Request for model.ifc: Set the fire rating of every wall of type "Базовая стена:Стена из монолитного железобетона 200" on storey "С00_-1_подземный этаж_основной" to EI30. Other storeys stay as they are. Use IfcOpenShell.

First a look at what the model holds.

```python
import ifcopenshell
import ifcopenshell.util.element

model = ifcopenshell.open("model.ifc")
print(model.schema)
storey = next(s for s in model.by_type("IfcBuildingStorey") if s.Name == "С00_-1_подземный этаж_основной")
walls = [e for e in ifcopenshell.util.element.get_decomposition(storey) if e.is_a("IfcWall")]
seen = {}
for e in walls:
    element_type = ifcopenshell.util.element.get_type(e)
    key = (element_type.Name if element_type != e and element_type else None, ifcopenshell.util.element.get_pset(e, "Pset_WallCommon", "FireRating"))
    seen[key] = seen.get(key, 0) + 1
for (name, value), count in sorted(seen.items(), key=str):
    print(count, "x", name, "|", value)
```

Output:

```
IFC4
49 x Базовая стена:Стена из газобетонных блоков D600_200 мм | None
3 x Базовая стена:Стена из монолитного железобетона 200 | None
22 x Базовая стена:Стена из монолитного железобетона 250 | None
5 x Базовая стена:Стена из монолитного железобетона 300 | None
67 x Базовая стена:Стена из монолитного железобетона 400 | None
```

```python
import ifcopenshell
import ifcopenshell.api.pset
import ifcopenshell.util.element

model = ifcopenshell.open("model.ifc")

storey = next(s for s in model.by_type("IfcBuildingStorey") if s.Name == "С00_-1_подземный этаж_основной")
walls = [e for e in ifcopenshell.util.element.get_decomposition(storey) if e.is_a("IfcWall")]

count = 0
for e in walls:
    element_type = ifcopenshell.util.element.get_type(e)
    if element_type in (None, e) or element_type.Name != "Базовая стена:Стена из монолитного железобетона 200":
        continue
    # add_pset returns the element's existing set when there is one.
    pset = ifcopenshell.api.pset.add_pset(model, product=e, name="Pset_WallCommon")
    ifcopenshell.api.pset.edit_pset(model, pset=pset, properties={"FireRating": "EI30"})
    count += 1

print(count, "walls updated")

model.write("model_v2.ifc")
```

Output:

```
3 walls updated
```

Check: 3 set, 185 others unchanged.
